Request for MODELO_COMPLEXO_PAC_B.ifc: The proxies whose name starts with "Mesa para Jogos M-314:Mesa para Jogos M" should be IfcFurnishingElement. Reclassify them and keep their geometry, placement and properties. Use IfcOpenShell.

First a look at what the model holds.

```python
import re

import ifcopenshell

model = ifcopenshell.open("MODELO_COMPLEXO_PAC_B.ifc")
print(model.schema)
seen = {}
for e in model.by_type("IfcBuildingElementProxy"):
    name = re.sub(r":\d+(:\d+)?$", "", e.Name or "")  # drop the element id that some exporters append
    seen[name] = seen.get(name, 0) + 1
for name, count in sorted(seen.items()):
    print(count, "x", name)
```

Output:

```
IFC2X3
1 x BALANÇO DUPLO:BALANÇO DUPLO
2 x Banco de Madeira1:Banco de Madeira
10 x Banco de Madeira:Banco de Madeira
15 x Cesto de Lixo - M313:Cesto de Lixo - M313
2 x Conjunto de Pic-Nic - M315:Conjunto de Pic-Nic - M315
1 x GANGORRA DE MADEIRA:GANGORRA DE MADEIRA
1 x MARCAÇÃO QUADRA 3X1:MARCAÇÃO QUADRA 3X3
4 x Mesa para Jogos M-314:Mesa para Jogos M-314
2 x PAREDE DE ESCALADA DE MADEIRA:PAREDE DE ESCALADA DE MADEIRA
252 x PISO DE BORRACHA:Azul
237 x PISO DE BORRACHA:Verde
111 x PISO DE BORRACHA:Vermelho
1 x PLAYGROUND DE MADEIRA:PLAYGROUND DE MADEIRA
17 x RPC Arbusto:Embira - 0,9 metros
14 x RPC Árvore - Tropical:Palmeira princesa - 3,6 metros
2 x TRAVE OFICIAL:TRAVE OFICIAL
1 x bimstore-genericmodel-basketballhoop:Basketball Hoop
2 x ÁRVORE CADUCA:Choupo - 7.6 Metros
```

```python
import ifcopenshell
import ifcopenshell.api.root

model = ifcopenshell.open("MODELO_COMPLEXO_PAC_B.ifc")

proxies = [e.id() for e in model.by_type("IfcBuildingElementProxy") if (e.Name or "").startswith("Mesa para Jogos M-314:Mesa para Jogos M")]
for step_id in proxies:
    proxy = model.by_id(step_id)
    # Reclassifying a typed element also reclassifies its type and the type's other occurrences.
    if proxy.is_a("IfcBuildingElementProxy"):
        ifcopenshell.api.root.reassign_class(model, product=proxy, ifc_class="IfcFurnishingElement")

print(sum(model.by_id(i).is_a("IfcFurnishingElement") for i in proxies), "reclassified")

model.write("MODELO_COMPLEXO_PAC_B_v2.ifc")
```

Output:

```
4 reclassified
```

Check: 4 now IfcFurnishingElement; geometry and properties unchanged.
